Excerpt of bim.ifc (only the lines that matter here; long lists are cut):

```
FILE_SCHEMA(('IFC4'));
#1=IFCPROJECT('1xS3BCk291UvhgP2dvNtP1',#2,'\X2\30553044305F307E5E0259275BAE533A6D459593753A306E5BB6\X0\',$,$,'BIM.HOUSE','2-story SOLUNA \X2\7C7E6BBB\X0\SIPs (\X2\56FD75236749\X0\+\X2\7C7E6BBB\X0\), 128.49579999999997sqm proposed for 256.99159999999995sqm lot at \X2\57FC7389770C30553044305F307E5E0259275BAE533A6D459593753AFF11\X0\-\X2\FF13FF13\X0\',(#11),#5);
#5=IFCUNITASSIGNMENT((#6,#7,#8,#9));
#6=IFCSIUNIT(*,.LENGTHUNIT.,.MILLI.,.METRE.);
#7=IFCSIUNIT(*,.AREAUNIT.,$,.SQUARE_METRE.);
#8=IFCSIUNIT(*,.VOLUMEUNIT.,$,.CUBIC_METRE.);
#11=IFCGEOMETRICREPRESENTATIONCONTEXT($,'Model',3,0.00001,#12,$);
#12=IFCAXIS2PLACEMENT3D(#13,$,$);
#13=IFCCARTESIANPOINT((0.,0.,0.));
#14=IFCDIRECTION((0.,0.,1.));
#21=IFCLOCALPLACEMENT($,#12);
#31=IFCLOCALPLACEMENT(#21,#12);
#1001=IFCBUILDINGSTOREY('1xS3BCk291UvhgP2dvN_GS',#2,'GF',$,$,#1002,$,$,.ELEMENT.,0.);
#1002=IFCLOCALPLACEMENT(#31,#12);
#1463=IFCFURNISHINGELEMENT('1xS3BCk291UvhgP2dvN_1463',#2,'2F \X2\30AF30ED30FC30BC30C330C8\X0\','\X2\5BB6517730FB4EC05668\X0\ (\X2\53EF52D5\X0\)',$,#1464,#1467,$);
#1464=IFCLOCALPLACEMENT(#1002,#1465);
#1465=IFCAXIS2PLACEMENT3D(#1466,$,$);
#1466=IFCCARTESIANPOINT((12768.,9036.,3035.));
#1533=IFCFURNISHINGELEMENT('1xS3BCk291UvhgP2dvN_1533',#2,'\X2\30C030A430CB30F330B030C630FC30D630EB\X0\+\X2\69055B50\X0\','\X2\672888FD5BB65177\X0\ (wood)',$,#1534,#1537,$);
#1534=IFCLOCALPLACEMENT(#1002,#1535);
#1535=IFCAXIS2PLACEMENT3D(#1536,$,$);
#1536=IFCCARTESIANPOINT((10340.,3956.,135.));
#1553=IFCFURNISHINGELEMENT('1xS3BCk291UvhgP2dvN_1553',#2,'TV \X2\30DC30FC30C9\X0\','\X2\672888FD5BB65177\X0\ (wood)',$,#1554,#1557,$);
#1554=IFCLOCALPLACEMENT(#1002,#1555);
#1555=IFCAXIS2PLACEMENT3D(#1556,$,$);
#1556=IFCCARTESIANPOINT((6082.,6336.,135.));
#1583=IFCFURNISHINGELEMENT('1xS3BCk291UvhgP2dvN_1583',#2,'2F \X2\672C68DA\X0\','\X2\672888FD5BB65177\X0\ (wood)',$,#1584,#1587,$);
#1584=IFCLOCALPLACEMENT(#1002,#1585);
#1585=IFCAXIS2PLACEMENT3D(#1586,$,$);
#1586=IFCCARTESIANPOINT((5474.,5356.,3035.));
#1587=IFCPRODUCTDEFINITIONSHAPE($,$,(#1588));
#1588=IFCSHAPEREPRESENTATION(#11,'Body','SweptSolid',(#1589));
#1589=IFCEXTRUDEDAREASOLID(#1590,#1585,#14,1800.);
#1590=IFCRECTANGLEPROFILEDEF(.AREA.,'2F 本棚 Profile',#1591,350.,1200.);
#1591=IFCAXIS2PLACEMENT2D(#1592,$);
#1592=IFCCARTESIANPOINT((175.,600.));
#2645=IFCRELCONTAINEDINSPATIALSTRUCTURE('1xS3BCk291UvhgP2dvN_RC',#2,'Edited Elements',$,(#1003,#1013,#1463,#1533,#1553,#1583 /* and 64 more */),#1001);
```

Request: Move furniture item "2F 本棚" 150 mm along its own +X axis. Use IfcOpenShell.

```python
import ifcopenshell
import ifcopenshell.api.geometry
import ifcopenshell.util.placement
import ifcopenshell.util.unit

model = ifcopenshell.open("bim.ifc")
unit_scale = ifcopenshell.util.unit.calculate_unit_scale(model)

item = model.by_guid("1xS3BCk291UvhgP2dvN_1583")
matrix = ifcopenshell.util.placement.get_local_placement(item.ObjectPlacement)
matrix[:3, 3] += matrix[:3, 0] * 0.15 / unit_scale
ifcopenshell.api.geometry.edit_object_placement(model, product=item, matrix=matrix, is_si=False)

print(ifcopenshell.util.placement.get_local_placement(item.ObjectPlacement).round(3) + 0.0)

model.write("bim_rev.ifc")
```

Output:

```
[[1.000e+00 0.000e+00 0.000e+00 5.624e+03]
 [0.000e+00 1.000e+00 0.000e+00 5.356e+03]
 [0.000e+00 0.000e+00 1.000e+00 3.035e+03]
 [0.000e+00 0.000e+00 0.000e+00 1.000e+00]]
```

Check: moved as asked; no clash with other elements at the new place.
